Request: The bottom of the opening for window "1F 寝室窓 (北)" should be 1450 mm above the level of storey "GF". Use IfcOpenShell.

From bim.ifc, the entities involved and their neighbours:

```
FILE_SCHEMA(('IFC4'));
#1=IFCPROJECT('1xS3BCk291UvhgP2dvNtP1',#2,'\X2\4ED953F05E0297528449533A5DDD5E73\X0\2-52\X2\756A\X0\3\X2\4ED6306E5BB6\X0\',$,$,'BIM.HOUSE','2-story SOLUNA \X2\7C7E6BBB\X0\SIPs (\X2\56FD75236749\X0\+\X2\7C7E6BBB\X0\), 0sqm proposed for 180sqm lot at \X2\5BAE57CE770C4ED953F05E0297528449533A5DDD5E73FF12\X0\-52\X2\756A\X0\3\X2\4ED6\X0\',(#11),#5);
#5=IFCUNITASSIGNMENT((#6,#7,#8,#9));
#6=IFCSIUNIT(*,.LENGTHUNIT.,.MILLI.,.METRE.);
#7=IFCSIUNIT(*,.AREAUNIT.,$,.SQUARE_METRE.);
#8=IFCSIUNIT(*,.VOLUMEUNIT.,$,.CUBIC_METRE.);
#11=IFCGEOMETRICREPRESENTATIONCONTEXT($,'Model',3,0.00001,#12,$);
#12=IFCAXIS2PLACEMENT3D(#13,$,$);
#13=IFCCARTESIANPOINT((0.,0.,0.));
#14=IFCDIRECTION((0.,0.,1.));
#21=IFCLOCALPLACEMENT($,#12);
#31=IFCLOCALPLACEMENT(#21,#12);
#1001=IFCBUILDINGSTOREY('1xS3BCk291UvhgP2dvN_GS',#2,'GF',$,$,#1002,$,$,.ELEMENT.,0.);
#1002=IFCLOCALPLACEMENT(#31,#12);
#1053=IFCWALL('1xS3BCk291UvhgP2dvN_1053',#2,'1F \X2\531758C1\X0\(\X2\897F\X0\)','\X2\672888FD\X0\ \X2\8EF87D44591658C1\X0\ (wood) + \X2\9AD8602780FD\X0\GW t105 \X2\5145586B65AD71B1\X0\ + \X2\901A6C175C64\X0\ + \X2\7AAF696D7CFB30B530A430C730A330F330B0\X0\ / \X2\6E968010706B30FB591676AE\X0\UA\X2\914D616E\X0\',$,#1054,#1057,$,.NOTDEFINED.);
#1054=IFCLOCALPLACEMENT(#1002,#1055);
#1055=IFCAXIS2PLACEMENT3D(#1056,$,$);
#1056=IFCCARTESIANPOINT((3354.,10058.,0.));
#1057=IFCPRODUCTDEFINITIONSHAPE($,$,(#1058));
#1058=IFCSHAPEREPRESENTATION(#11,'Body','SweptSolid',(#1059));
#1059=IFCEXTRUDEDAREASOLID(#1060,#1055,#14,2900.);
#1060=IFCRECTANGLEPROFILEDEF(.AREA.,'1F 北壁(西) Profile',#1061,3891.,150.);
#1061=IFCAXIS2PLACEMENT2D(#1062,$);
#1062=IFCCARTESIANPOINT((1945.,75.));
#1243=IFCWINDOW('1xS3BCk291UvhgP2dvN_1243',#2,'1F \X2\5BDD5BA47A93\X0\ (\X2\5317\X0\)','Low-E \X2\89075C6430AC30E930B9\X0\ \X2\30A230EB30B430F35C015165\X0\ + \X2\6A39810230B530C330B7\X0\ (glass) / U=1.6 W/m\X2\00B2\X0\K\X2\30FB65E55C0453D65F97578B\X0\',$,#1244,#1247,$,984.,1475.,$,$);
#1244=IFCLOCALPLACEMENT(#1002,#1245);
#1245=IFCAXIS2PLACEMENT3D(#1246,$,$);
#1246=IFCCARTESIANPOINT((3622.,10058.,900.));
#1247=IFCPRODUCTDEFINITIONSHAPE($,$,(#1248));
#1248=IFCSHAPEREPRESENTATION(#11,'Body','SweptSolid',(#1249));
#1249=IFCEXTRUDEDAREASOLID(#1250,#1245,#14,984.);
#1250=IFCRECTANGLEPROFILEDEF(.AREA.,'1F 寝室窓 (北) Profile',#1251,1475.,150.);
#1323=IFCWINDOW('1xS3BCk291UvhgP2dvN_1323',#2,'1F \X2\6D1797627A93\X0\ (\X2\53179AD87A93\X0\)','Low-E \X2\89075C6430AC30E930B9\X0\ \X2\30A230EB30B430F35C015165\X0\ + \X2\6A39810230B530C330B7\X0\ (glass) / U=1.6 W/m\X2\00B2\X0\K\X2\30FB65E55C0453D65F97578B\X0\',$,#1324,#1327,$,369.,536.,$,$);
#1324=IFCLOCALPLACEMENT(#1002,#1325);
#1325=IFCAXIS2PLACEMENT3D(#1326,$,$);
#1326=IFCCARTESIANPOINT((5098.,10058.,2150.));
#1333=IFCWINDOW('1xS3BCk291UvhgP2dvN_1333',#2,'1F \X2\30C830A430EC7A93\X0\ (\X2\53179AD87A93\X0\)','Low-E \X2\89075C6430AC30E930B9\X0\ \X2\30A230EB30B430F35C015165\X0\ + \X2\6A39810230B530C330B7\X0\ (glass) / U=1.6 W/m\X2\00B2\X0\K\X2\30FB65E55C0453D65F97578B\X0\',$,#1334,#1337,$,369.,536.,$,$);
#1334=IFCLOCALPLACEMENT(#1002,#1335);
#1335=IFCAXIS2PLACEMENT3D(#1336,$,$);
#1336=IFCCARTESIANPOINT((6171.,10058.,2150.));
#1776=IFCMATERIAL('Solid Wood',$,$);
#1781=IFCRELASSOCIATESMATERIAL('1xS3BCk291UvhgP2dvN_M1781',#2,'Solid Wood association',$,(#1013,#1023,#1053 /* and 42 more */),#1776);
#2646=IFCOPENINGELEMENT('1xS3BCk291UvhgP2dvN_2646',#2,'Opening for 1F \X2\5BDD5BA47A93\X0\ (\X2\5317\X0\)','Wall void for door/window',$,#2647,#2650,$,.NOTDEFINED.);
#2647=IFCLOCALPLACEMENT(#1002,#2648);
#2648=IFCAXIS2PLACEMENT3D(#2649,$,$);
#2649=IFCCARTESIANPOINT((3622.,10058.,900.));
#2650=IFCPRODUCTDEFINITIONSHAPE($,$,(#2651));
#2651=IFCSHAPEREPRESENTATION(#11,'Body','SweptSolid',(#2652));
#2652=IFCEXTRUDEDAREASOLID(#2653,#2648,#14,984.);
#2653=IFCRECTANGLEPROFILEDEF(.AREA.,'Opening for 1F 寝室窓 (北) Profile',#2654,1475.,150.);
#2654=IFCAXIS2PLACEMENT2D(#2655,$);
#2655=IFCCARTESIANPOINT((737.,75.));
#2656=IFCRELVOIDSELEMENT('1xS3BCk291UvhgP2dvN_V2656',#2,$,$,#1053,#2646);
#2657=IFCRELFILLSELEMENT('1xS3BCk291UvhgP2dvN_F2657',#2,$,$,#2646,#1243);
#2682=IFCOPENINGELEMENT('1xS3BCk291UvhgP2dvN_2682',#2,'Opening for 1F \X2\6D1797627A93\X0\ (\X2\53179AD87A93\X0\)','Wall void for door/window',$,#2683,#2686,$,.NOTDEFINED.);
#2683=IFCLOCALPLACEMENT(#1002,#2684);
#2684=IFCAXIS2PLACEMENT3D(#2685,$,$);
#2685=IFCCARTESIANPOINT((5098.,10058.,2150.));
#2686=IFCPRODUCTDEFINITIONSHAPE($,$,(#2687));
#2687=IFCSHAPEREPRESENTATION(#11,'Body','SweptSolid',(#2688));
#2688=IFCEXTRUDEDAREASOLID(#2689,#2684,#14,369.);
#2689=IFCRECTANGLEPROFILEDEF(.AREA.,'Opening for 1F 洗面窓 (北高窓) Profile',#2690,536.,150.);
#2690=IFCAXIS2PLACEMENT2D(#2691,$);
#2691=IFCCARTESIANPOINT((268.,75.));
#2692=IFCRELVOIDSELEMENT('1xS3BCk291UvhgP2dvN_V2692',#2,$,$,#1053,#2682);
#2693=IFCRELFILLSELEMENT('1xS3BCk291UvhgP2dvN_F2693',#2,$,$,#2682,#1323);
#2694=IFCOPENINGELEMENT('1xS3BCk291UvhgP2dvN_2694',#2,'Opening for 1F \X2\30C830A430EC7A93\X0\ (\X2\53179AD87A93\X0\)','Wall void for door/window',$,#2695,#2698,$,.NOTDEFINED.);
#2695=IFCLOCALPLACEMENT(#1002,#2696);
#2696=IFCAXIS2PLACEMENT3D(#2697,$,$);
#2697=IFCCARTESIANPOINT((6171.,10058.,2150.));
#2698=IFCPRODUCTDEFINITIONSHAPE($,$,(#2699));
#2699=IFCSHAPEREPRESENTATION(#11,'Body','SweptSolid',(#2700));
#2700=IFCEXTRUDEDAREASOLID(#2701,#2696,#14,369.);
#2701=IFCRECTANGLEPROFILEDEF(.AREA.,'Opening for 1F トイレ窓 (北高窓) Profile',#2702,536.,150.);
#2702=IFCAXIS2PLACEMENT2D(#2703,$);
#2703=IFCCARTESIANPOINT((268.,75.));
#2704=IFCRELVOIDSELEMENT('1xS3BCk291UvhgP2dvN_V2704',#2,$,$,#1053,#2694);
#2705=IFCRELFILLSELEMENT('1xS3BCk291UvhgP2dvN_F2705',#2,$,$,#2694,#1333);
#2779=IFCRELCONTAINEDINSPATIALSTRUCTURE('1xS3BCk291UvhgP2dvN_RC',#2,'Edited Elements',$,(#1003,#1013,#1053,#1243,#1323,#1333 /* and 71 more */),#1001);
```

```python
import numpy as np
import ifcopenshell
import ifcopenshell.api.geometry
import ifcopenshell.geom
import ifcopenshell.util.element
import ifcopenshell.util.placement
import ifcopenshell.util.shape
import ifcopenshell.util.unit

model = ifcopenshell.open("bim.ifc")
unit_scale = ifcopenshell.util.unit.calculate_unit_scale(model)

window = model.by_id(1243)
opening = window.FillsVoids[0].RelatingOpeningElement
storey = ifcopenshell.util.element.get_container(window, ifc_class="IfcBuildingStorey")
level = ifcopenshell.util.placement.get_local_placement(storey.ObjectPlacement)[2, 3]

# The opening's origin need not be at the sill, so measure its lowest point.
shape = ifcopenshell.geom.create_shape(ifcopenshell.geom.settings(), opening)
bottom = ifcopenshell.util.shape.get_shape_bottom_elevation(shape, shape.geometry) / unit_scale
dz = level + 1450.0 - bottom

shift = np.array([0.0, 0.0, dz])
# The window is not placed relative to its opening, so move both.
for product in (opening, window):
    matrix = ifcopenshell.util.placement.get_local_placement(product.ObjectPlacement)
    matrix[:3, 3] += shift
    ifcopenshell.api.geometry.edit_object_placement(model, product=product, matrix=matrix, is_si=False)

print(f"moved by {dz * unit_scale:+.3f} m")

model.write("bim_edited.ifc")
```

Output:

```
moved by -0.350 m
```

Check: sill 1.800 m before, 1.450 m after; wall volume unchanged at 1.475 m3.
